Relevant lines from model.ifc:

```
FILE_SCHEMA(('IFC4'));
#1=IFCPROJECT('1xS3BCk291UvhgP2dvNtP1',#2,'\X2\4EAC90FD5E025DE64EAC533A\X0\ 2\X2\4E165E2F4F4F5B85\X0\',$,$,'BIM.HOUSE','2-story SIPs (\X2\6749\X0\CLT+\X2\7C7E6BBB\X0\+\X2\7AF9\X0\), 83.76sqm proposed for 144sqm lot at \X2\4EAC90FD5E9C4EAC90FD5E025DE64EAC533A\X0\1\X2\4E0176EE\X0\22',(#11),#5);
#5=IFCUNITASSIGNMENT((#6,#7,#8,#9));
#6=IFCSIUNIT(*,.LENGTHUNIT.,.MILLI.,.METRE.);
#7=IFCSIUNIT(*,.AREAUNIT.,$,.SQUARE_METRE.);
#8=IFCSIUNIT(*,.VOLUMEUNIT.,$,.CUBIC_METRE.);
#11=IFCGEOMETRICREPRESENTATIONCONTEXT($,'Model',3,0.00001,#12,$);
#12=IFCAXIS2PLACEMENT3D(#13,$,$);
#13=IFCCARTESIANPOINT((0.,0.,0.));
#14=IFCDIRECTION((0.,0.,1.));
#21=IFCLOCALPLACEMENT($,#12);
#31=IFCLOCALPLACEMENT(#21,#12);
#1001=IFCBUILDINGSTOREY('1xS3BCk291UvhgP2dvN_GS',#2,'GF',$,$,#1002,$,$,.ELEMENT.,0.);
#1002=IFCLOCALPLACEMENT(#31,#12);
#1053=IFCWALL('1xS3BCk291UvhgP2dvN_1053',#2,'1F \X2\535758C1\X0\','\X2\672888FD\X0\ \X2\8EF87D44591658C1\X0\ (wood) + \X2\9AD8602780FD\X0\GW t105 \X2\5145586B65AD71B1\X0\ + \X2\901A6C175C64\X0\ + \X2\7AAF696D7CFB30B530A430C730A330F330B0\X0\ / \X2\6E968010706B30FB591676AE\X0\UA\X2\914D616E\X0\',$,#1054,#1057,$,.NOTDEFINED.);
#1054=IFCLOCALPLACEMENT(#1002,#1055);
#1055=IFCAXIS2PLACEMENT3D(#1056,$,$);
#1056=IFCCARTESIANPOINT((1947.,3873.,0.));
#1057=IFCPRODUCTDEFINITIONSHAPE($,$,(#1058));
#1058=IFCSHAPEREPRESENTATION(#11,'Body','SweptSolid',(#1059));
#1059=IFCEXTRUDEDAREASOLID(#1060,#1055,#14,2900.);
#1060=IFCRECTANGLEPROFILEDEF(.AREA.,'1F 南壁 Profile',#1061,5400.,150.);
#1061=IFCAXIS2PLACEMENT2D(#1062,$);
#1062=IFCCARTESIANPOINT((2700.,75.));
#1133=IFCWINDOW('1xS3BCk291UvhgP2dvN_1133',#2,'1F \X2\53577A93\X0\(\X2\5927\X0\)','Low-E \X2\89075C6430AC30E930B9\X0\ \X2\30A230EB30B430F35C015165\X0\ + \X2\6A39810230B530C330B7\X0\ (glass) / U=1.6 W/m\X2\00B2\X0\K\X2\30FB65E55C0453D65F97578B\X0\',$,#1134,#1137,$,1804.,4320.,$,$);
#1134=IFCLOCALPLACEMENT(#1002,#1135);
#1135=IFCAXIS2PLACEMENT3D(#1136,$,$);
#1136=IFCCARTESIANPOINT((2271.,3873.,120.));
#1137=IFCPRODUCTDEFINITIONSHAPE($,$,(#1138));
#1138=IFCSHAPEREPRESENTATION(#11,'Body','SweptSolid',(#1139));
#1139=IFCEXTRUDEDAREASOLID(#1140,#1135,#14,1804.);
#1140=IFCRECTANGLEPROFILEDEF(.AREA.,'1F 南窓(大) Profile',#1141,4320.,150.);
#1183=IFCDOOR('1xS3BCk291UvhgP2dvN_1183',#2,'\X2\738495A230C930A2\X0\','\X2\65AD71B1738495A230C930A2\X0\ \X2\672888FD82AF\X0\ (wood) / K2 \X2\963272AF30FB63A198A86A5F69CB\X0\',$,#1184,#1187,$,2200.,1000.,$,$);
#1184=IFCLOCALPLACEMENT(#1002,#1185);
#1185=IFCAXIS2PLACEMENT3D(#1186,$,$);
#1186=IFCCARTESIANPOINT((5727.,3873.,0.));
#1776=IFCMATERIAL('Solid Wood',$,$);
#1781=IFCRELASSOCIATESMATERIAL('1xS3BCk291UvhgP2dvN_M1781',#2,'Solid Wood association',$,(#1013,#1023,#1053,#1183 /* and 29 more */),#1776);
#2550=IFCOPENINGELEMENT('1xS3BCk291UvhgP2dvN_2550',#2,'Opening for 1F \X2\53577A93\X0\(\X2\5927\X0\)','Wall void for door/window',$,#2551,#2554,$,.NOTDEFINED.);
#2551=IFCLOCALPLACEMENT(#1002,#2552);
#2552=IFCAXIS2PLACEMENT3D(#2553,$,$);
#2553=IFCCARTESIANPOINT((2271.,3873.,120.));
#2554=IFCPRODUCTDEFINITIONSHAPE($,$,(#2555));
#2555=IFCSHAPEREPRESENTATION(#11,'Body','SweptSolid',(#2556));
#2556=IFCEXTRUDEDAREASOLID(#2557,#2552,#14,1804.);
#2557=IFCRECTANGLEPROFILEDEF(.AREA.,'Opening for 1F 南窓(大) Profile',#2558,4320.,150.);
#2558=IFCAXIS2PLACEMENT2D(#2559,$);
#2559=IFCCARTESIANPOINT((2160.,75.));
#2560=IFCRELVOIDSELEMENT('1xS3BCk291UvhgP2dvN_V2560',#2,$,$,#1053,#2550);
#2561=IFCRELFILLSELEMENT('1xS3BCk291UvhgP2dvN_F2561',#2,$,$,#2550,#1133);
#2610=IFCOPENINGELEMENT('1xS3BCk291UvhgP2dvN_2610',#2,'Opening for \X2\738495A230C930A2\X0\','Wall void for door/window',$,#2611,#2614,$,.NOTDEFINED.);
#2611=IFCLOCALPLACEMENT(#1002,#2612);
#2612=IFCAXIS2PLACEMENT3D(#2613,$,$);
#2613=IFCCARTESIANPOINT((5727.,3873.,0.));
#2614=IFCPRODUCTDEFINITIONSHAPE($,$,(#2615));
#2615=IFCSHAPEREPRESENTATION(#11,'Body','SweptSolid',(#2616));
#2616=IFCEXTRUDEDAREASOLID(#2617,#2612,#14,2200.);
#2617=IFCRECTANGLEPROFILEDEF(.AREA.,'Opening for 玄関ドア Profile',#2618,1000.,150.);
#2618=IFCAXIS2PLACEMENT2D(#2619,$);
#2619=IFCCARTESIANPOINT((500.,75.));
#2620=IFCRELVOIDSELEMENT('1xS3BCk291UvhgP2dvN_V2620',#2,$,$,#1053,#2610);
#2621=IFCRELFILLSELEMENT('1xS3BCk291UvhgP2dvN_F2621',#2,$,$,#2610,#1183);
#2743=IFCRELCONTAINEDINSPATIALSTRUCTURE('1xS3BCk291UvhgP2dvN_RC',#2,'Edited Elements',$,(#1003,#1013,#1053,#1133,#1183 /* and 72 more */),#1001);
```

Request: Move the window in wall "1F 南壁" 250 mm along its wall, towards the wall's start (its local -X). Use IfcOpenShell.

```python
import ifcopenshell
import ifcopenshell.api.geometry
import ifcopenshell.util.placement

model = ifcopenshell.open("model.ifc")

window = model.by_guid("1xS3BCk291UvhgP2dvN_1133")
opening = window.FillsVoids[0].RelatingOpeningElement
wall = opening.VoidsElements[0].RelatingBuildingElement

wall_matrix = ifcopenshell.util.placement.get_local_placement(wall.ObjectPlacement)
shift = wall_matrix[:3, 0] * -250.0
before = ifcopenshell.util.placement.get_local_placement(window.ObjectPlacement)[:3, 3].copy()

# The window is not placed relative to its opening, so move both.
for product in (opening, window):
    matrix = ifcopenshell.util.placement.get_local_placement(product.ObjectPlacement)
    matrix[:3, 3] += shift
    ifcopenshell.api.geometry.edit_object_placement(model, product=product, matrix=matrix, is_si=False)

after = ifcopenshell.util.placement.get_local_placement(window.ObjectPlacement)[:3, 3]
print("window moved by", (after - before).round(3) + 0.0)

model.write("model_edited.ifc")
```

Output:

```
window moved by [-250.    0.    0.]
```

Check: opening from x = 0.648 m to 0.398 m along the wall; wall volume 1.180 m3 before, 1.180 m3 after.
